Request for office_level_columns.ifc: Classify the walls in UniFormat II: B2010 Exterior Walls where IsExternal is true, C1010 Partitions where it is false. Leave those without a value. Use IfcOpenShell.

First a look at what the model holds.

```python
import ifcopenshell
import ifcopenshell.util.element

model = ifcopenshell.open("office_level_columns.ifc")
print(model.schema)
print("classifications:", [c.Name for c in model.by_type("IfcClassification")])
values = [ifcopenshell.util.element.get_pset(e, "Pset_WallCommon", "IsExternal") for e in model.by_type("IfcWall")]
for value in (True, False, None):
    print("IsExternal", value, values.count(value))
```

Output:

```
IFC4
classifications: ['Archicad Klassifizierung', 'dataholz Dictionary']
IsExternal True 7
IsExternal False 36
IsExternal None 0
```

```python
import ifcopenshell
import ifcopenshell.api.classification
import ifcopenshell.util.element

model = ifcopenshell.open("office_level_columns.ifc")

system = ifcopenshell.api.classification.add_classification(model, classification="UniFormat II")

walls = model.by_type("IfcWall")
external = {e: ifcopenshell.util.element.get_pset(e, "Pset_WallCommon", "IsExternal") for e in walls}
for flag, code, name in ((True, "B2010", "Exterior Walls"), (False, "C1010", "Partitions")):
    products = [e for e in walls if external[e] is flag]
    ifcopenshell.api.classification.add_reference(
        model, products=products, classification=system, identification=code, name=name
    )
    print(code, len(products))

model.write("office_level_columns_updated.ifc")
```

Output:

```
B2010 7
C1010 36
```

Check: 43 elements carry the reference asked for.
